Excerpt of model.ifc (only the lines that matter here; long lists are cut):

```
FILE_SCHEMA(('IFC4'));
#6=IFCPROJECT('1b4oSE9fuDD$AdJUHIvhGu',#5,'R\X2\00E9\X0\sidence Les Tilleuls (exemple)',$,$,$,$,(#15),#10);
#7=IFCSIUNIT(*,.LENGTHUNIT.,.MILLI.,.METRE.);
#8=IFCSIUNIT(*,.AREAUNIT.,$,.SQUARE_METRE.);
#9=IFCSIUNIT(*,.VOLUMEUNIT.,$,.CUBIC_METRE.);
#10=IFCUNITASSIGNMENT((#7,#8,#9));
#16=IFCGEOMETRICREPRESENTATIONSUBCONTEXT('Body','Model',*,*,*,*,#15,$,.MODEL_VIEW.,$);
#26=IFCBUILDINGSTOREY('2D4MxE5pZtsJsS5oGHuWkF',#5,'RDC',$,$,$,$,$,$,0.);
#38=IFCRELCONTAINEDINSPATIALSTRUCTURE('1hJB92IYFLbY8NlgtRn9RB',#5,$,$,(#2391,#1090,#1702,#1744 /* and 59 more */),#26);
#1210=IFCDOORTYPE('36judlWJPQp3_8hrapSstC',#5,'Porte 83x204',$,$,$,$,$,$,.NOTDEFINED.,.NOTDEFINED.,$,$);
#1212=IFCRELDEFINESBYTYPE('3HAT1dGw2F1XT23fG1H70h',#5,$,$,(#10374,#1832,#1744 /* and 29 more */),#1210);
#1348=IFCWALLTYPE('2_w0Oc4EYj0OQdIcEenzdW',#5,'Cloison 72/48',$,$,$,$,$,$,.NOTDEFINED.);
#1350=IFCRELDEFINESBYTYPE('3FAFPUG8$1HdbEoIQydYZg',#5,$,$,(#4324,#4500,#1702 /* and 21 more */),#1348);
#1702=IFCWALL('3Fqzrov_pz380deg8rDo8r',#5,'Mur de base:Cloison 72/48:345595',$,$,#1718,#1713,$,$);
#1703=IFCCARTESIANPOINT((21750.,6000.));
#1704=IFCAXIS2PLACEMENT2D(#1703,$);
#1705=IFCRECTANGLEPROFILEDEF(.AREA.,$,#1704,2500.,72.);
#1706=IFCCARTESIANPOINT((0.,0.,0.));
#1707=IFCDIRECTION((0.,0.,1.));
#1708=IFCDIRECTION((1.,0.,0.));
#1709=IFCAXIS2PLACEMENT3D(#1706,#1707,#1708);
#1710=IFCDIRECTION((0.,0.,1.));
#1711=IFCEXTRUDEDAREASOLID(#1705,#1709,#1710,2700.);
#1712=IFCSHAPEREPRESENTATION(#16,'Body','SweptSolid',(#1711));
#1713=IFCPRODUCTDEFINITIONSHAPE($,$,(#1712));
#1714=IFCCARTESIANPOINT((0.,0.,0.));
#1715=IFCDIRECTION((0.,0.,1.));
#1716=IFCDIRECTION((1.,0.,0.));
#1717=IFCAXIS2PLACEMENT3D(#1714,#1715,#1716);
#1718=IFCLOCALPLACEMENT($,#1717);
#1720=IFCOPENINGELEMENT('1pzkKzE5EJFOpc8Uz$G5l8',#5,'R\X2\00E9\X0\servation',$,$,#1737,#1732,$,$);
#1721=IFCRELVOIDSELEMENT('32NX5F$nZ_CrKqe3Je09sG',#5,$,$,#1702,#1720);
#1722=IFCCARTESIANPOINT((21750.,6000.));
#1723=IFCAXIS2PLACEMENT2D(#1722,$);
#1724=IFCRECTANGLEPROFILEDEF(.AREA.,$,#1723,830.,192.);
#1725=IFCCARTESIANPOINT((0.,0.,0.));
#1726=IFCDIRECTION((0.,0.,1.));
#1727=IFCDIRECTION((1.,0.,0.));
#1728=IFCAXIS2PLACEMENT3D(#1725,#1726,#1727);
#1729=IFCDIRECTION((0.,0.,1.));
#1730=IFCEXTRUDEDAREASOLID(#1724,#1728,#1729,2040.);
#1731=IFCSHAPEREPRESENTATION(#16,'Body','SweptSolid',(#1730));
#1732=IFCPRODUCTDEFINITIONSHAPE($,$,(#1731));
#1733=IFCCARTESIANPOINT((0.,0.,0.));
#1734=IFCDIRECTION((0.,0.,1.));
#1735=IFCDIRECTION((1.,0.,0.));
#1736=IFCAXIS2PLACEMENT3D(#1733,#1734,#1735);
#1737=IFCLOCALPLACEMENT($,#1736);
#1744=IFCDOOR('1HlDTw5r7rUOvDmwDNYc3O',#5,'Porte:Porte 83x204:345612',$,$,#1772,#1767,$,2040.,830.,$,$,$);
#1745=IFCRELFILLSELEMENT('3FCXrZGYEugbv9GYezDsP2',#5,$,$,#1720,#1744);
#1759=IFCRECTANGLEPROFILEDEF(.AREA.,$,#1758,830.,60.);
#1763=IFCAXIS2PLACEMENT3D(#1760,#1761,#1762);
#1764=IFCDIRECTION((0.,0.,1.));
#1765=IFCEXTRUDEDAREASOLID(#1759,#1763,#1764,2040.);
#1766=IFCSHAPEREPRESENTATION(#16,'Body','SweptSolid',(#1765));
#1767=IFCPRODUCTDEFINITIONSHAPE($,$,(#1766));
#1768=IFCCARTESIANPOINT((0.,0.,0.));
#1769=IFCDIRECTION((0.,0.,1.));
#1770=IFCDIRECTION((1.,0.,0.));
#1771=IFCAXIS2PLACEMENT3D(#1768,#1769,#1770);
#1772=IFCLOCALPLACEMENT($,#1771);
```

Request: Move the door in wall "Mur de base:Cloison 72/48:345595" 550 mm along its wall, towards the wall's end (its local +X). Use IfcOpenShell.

```python
import ifcopenshell
import ifcopenshell.api.geometry
import ifcopenshell.util.placement
import ifcopenshell.util.unit

model = ifcopenshell.open("model.ifc")
unit_scale = ifcopenshell.util.unit.calculate_unit_scale(model)

door = model.by_guid("1HlDTw5r7rUOvDmwDNYc3O")
opening = door.FillsVoids[0].RelatingOpeningElement
wall = opening.VoidsElements[0].RelatingBuildingElement

wall_matrix = ifcopenshell.util.placement.get_local_placement(wall.ObjectPlacement)
shift = wall_matrix[:3, 0] * 0.55 / unit_scale
before = ifcopenshell.util.placement.get_local_placement(door.ObjectPlacement)[:3, 3].copy()

# The door is not placed relative to its opening, so move both.
for product in (opening, door):
    matrix = ifcopenshell.util.placement.get_local_placement(product.ObjectPlacement)
    matrix[:3, 3] += shift
    ifcopenshell.api.geometry.edit_object_placement(model, product=product, matrix=matrix, is_si=False)

after = ifcopenshell.util.placement.get_local_placement(door.ObjectPlacement)[:3, 3]
print("door moved by", (after - before).round(3) + 0.0)

model.write("model_rev.ifc")
```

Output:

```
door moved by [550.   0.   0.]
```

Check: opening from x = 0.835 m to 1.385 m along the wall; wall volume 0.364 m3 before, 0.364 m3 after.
